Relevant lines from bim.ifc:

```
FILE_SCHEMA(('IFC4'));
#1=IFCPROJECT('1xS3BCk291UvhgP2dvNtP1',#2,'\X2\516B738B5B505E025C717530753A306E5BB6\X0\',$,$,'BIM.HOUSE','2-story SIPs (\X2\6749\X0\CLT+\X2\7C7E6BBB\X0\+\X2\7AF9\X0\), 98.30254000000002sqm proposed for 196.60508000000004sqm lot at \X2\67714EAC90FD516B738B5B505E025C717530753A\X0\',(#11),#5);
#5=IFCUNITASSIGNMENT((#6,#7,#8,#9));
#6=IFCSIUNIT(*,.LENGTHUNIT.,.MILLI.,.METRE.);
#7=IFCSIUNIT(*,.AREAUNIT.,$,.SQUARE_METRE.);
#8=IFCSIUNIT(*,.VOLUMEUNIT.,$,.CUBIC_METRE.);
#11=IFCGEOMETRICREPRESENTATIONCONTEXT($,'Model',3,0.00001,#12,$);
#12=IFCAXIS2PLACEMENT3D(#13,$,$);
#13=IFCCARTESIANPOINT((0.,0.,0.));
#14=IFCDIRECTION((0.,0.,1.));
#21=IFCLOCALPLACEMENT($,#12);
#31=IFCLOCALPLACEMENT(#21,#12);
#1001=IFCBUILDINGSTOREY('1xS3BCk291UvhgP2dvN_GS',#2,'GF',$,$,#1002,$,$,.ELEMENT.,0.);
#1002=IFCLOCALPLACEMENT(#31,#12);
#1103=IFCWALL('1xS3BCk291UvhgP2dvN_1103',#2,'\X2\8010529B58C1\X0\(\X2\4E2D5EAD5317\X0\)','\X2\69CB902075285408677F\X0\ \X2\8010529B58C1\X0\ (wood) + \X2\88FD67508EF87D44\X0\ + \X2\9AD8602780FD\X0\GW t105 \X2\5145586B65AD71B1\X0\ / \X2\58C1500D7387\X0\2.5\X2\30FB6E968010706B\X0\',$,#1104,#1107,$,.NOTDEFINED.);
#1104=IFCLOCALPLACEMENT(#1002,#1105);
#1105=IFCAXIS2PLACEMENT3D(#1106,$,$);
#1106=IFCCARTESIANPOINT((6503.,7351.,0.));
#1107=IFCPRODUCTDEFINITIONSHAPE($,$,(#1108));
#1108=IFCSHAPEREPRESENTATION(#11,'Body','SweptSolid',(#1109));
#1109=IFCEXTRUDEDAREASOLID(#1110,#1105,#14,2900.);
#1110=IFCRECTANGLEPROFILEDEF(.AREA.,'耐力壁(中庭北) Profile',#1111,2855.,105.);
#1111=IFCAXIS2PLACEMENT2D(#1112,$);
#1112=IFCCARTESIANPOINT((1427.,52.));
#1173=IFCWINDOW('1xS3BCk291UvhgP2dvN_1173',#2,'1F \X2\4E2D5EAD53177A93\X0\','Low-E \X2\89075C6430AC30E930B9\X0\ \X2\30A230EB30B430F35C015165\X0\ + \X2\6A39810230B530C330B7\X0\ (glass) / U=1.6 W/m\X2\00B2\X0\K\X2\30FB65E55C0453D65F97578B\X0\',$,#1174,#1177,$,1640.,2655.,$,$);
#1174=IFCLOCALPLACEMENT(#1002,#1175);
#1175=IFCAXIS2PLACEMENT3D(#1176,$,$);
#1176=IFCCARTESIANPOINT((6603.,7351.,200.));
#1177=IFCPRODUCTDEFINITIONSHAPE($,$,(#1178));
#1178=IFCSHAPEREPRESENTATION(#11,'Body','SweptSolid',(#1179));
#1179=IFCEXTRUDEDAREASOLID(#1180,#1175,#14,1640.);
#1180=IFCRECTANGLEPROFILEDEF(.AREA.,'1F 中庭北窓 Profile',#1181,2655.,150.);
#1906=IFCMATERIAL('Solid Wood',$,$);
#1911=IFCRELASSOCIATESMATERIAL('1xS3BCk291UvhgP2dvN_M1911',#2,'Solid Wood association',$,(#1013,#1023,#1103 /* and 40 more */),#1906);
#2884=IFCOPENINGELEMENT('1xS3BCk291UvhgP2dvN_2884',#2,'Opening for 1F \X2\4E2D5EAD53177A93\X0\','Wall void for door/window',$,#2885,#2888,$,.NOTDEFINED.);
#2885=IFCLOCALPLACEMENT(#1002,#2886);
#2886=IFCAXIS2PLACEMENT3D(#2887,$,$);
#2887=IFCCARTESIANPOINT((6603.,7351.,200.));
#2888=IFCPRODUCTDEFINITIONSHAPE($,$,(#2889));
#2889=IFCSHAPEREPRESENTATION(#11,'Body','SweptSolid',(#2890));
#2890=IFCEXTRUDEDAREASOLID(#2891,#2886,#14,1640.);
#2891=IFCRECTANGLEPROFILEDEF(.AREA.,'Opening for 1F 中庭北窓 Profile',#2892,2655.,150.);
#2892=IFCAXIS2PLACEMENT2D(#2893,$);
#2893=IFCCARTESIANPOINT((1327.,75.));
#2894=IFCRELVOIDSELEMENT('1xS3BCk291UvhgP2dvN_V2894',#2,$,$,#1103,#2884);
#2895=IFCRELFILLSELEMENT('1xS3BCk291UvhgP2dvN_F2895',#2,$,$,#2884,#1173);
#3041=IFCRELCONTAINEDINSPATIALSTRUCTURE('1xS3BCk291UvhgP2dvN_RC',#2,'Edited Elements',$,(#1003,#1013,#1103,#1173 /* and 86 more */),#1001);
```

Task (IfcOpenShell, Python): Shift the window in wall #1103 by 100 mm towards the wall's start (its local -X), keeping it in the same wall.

```python
import ifcopenshell
import ifcopenshell.api.geometry
import ifcopenshell.util.placement

model = ifcopenshell.open("bim.ifc")

window = model.by_guid("1xS3BCk291UvhgP2dvN_1173")
opening = window.FillsVoids[0].RelatingOpeningElement
wall = opening.VoidsElements[0].RelatingBuildingElement

wall_matrix = ifcopenshell.util.placement.get_local_placement(wall.ObjectPlacement)
shift = wall_matrix[:3, 0] * -100.0
before = ifcopenshell.util.placement.get_local_placement(window.ObjectPlacement)[:3, 3].copy()

# The window is not placed relative to its opening, so move both.
for product in (opening, window):
    matrix = ifcopenshell.util.placement.get_local_placement(product.ObjectPlacement)
    matrix[:3, 3] += shift
    ifcopenshell.api.geometry.edit_object_placement(model, product=product, matrix=matrix, is_si=False)

after = ifcopenshell.util.placement.get_local_placement(window.ObjectPlacement)[:3, 3]
print("window moved by", (after - before).round(3) + 0.0)

model.write("bim_rev.ifc")
```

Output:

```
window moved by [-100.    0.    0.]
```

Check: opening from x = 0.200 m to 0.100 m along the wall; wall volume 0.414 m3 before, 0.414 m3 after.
